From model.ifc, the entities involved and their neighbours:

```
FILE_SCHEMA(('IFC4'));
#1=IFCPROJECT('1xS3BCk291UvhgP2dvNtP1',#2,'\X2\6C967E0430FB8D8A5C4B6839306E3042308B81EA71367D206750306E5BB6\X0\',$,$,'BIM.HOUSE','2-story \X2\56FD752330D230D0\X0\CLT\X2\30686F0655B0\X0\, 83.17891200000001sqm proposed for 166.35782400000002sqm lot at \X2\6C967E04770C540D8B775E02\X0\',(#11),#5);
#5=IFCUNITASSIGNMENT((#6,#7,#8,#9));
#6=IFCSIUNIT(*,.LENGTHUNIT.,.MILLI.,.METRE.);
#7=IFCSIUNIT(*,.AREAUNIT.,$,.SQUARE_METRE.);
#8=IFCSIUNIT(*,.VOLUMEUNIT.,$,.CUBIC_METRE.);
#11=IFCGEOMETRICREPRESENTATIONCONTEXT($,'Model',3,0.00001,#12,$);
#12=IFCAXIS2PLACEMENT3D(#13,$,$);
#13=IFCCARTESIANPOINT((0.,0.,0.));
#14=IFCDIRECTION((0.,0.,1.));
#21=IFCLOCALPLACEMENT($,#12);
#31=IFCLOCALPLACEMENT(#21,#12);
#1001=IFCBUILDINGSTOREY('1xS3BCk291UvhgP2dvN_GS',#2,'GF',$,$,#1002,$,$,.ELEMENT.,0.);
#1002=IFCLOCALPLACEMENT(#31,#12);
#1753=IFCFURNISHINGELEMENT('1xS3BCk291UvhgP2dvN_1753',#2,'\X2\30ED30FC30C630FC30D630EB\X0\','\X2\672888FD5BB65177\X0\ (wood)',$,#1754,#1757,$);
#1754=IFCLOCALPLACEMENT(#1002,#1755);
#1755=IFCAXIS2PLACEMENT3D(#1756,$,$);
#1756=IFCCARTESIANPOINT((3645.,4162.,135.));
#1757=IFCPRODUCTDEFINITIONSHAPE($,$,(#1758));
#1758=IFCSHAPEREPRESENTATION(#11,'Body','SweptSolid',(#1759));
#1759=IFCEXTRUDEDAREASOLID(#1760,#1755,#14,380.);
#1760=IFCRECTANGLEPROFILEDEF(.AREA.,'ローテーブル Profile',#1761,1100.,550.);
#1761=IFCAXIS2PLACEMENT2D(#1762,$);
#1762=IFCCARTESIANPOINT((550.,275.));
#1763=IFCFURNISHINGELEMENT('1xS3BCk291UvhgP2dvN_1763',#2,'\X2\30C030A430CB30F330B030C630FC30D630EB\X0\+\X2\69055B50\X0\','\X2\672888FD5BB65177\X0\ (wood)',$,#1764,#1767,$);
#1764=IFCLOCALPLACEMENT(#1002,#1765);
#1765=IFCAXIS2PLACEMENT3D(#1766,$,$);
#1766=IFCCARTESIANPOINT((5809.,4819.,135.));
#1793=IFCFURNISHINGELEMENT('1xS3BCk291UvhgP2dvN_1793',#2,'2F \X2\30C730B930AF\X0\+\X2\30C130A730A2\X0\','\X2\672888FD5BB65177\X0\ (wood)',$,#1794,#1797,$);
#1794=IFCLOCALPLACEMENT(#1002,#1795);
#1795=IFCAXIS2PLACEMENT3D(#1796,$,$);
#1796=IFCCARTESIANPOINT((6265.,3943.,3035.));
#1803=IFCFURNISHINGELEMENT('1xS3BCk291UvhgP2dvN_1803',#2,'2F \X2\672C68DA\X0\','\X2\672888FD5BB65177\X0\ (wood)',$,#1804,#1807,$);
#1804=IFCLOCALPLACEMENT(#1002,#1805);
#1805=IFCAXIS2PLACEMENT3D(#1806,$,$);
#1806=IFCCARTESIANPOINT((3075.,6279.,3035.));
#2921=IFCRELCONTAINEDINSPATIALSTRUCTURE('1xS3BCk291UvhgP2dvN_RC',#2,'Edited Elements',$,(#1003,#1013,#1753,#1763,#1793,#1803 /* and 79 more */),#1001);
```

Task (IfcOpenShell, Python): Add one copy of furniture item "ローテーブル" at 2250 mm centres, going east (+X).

```python
import numpy as np
import ifcopenshell
import ifcopenshell.api.geometry
import ifcopenshell.api.root
import ifcopenshell.util.element
import ifcopenshell.util.placement
import ifcopenshell.util.unit

model = ifcopenshell.open("model.ifc")
unit_scale = ifcopenshell.util.unit.calculate_unit_scale(model)


def reuse_history(source, copy):
    """copy_class also copies each property set's owner history, people and application; keep the originals."""
    for rel in copy.IsDefinedBy:
        if rel.is_a("IfcRelDefinesByProperties") and (history := rel.RelatingPropertyDefinition.OwnerHistory):
            rel.RelatingPropertyDefinition.OwnerHistory = source.OwnerHistory
            ifcopenshell.util.element.remove_deep2(model, history)


source = model.by_guid("1xS3BCk291UvhgP2dvN_1753")
base = ifcopenshell.util.placement.get_local_placement(source.ObjectPlacement)
step = np.array([1.0, 0.0, 0.0]) * 2.25 / unit_scale

for i in range(1, 2):
    copy = ifcopenshell.api.root.copy_class(model, product=source)
    copy.Representation = ifcopenshell.util.element.copy_deep(
        model, source.Representation, exclude=["IfcGeometricRepresentationContext", "IfcRepresentationMap"]
    )
    reuse_history(source, copy)
    matrix = base.copy()
    matrix[:3, 3] += i * step
    print("added at", matrix[:3, 3].round(3) + 0.0)
    ifcopenshell.api.geometry.edit_object_placement(model, product=copy, matrix=matrix, is_si=False)

model.write("model-out.ifc")
```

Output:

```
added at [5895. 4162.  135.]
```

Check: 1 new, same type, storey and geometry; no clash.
